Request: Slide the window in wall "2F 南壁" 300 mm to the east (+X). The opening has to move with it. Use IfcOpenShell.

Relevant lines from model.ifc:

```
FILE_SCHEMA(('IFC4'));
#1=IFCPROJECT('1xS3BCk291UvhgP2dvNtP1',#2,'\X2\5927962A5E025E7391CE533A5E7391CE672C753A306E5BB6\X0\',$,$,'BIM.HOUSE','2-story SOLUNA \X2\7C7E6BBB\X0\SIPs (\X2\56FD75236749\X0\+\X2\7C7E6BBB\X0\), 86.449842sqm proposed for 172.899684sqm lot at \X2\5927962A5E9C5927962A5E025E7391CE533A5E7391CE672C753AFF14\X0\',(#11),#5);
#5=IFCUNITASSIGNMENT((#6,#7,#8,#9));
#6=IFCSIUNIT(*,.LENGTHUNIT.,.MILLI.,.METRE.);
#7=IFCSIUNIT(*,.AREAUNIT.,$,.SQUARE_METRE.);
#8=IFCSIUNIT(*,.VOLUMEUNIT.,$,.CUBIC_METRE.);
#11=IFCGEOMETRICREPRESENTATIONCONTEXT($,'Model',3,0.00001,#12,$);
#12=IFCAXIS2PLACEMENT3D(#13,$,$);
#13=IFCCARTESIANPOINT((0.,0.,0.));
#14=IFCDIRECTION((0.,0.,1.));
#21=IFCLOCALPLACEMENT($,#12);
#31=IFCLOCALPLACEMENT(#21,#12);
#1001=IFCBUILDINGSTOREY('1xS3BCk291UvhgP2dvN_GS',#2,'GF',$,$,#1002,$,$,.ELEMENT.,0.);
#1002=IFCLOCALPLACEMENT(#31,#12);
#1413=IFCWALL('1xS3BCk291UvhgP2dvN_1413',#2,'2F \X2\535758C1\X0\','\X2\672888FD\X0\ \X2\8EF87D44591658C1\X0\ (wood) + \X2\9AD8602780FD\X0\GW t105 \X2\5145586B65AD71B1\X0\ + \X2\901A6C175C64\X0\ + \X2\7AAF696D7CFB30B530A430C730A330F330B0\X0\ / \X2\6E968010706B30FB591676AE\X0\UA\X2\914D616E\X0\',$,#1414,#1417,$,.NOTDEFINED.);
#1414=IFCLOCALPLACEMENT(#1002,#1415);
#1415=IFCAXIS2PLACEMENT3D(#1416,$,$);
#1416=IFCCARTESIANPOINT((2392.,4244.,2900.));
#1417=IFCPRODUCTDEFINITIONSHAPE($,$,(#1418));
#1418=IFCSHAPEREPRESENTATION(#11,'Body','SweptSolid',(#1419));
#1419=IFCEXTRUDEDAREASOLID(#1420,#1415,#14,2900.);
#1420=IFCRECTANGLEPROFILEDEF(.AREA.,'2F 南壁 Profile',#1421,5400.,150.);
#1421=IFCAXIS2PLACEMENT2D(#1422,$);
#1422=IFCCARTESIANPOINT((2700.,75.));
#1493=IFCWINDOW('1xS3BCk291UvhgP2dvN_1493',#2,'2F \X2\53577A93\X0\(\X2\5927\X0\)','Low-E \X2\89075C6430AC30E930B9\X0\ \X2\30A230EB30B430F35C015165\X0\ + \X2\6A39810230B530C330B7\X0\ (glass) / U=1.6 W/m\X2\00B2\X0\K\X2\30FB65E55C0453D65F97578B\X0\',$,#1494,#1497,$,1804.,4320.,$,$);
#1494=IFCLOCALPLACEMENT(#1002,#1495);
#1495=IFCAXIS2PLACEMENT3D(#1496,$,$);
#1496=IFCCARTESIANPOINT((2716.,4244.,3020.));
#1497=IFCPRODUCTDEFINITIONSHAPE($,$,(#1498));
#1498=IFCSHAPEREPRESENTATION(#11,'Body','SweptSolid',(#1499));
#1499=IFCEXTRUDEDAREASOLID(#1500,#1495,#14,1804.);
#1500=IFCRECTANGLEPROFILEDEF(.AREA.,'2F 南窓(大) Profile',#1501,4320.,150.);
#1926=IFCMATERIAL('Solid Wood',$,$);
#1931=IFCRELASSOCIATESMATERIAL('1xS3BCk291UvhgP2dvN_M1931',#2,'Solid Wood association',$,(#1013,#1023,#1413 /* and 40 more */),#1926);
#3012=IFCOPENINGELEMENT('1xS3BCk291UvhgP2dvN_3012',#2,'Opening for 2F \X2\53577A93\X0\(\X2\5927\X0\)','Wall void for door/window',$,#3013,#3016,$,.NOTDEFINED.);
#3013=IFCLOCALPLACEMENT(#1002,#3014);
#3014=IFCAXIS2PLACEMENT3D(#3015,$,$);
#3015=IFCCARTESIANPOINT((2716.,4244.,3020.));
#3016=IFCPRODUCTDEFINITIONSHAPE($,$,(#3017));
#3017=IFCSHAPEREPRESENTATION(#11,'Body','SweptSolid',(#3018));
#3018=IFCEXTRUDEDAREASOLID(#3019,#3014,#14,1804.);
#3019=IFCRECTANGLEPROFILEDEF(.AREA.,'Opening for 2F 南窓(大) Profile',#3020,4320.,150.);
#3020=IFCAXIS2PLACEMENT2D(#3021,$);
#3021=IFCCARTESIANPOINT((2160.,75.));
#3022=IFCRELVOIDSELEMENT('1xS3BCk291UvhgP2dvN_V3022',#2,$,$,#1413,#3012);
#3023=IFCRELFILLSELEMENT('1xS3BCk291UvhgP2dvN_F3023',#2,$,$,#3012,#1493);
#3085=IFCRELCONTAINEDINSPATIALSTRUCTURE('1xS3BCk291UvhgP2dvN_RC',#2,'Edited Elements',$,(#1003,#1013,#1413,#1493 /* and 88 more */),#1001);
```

```python
import ifcopenshell
import ifcopenshell.api.geometry
import ifcopenshell.util.placement
import ifcopenshell.util.unit

model = ifcopenshell.open("model.ifc")
unit_scale = ifcopenshell.util.unit.calculate_unit_scale(model)

window = model.by_id(1493)
opening = window.FillsVoids[0].RelatingOpeningElement
wall = opening.VoidsElements[0].RelatingBuildingElement

wall_matrix = ifcopenshell.util.placement.get_local_placement(wall.ObjectPlacement)
shift = wall_matrix[:3, 0] * 0.3 / unit_scale
before = ifcopenshell.util.placement.get_local_placement(window.ObjectPlacement)[:3, 3].copy()

# The window is not placed relative to its opening, so move both.
for product in (opening, window):
    matrix = ifcopenshell.util.placement.get_local_placement(product.ObjectPlacement)
    matrix[:3, 3] += shift
    ifcopenshell.api.geometry.edit_object_placement(model, product=product, matrix=matrix, is_si=False)

after = ifcopenshell.util.placement.get_local_placement(window.ObjectPlacement)[:3, 3]
print("window moved by", (after - before).round(3) + 0.0)

model.write("model_v2.ifc")
```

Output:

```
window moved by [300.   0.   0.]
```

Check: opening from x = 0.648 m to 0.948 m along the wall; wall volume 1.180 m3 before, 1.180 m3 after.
